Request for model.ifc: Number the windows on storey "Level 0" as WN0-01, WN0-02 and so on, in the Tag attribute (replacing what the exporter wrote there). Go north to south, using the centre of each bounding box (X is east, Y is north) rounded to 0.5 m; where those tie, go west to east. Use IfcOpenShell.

First a look at what the model holds.

```python
import ifcopenshell
import ifcopenshell.util.element
import ifcopenshell.util.placement

model = ifcopenshell.open("model.ifc")
print(model.schema)
storey = next(s for s in model.by_type("IfcBuildingStorey") if s.Name == "Level 0")
windows = [e for e in ifcopenshell.util.element.get_decomposition(storey) if e.is_a("IfcWindow")]
for e in sorted(windows, key=lambda e: e.id()):
    origin = ifcopenshell.util.placement.get_local_placement(e.ObjectPlacement)[:3, 3]
    print(e.id(), e.Tag, e.Name, origin.round(2) + 0.0, sep=" | ")
```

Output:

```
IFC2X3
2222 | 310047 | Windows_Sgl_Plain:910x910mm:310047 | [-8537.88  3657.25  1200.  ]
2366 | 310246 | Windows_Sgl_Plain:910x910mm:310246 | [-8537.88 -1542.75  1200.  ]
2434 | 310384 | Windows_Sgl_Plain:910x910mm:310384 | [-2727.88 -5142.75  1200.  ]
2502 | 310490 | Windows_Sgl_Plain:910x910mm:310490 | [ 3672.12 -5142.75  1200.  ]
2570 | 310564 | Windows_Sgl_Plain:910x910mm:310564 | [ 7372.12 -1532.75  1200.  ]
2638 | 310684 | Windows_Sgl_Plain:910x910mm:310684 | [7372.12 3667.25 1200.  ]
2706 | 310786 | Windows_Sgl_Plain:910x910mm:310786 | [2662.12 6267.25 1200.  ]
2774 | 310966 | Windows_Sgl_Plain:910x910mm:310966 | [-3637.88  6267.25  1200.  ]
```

```python
import ifcopenshell
import ifcopenshell.geom
import ifcopenshell.util.element
import ifcopenshell.util.shape

model = ifcopenshell.open("model.ifc")
settings = ifcopenshell.geom.settings()
settings.set("use-world-coords", True)


def centre(element):
    shape = ifcopenshell.geom.create_shape(settings, element)
    return ifcopenshell.util.shape.get_bbox_centroid(shape.geometry)


storey = next(s for s in model.by_type("IfcBuildingStorey") if s.Name == "Level 0")
windows = [e for e in ifcopenshell.util.element.get_decomposition(storey) if e.is_a("IfcWindow")]

# Insertion points can sit at a corner or the storey origin, so sort by the geometry (in metres).
centres = {e: centre(e) for e in windows}
windows.sort(key=lambda e: (-round(centres[e][1] / 0.5), centres[e][0]))

for i, e in enumerate(windows, start=1):
    number = f"WN0-{i:02d}"
    e.Tag = number
    print(e.id(), number)

model.write("model_edited.ifc")
```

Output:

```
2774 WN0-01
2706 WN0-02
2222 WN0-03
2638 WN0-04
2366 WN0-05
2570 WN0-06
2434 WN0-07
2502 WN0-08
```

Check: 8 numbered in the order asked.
